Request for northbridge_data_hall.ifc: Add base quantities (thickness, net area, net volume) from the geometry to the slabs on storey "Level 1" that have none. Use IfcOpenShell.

First a look at what the model holds.

```python
import ifcopenshell
import ifcopenshell.util.element
import ifcopenshell.util.unit

model = ifcopenshell.open("northbridge_data_hall.ifc")
print(model.schema)
for unit_type in ("LENGTHUNIT", "AREAUNIT", "VOLUMEUNIT"):
    print(unit_type, ifcopenshell.util.unit.calculate_unit_scale(model, unit_type))
storey = next(s for s in model.by_type("IfcBuildingStorey") if s.Name == "Level 1")
slabs = [e for e in ifcopenshell.util.element.get_decomposition(storey) if e.is_a("IfcSlab")]
for e in sorted(slabs, key=lambda e: e.id()):
    print(e.id(), e.is_a(), e.Name, list(ifcopenshell.util.element.get_psets(e, qtos_only=True)), sep=" | ")
```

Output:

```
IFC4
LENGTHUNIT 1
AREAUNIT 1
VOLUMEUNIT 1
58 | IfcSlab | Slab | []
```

```python
import ifcopenshell
import ifcopenshell.api.pset
import ifcopenshell.geom
import ifcopenshell.util.element
import ifcopenshell.util.shape
import ifcopenshell.util.unit

model = ifcopenshell.open("northbridge_data_hall.ifc")
unit_scale = ifcopenshell.util.unit.calculate_unit_scale(model)
area_scale = ifcopenshell.util.unit.calculate_unit_scale(model, "AREAUNIT")
volume_scale = ifcopenshell.util.unit.calculate_unit_scale(model, "VOLUMEUNIT")
settings = ifcopenshell.geom.settings()

storey = next(s for s in model.by_type("IfcBuildingStorey") if s.Name == "Level 1")
slabs = [e for e in ifcopenshell.util.element.get_decomposition(storey) if e.is_a("IfcSlab")]

for e in sorted(slabs, key=lambda e: e.id()):
    if ifcopenshell.util.element.get_psets(e, qtos_only=True, should_inherit=False):
        continue
    # Geometry comes back in metres, in the element's own axes.
    shape = ifcopenshell.geom.create_shape(settings, e)
    values = {
        "Width": ifcopenshell.util.shape.get_z(shape.geometry) / unit_scale,
        "NetArea": ifcopenshell.util.shape.get_footprint_area(shape.geometry) / area_scale,
        "NetVolume": ifcopenshell.util.shape.get_volume(shape.geometry) / volume_scale,
    }
    qto = ifcopenshell.api.pset.add_qto(model, product=e, name="Qto_SlabBaseQuantities")
    ifcopenshell.api.pset.edit_qto(model, qto=qto, properties=values)
    print(e.id(), {k: round(v, 3) for k, v in values.items()})

model.write("northbridge_data_hall-out.ifc")
```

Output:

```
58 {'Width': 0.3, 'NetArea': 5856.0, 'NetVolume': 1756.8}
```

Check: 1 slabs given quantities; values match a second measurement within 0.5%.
